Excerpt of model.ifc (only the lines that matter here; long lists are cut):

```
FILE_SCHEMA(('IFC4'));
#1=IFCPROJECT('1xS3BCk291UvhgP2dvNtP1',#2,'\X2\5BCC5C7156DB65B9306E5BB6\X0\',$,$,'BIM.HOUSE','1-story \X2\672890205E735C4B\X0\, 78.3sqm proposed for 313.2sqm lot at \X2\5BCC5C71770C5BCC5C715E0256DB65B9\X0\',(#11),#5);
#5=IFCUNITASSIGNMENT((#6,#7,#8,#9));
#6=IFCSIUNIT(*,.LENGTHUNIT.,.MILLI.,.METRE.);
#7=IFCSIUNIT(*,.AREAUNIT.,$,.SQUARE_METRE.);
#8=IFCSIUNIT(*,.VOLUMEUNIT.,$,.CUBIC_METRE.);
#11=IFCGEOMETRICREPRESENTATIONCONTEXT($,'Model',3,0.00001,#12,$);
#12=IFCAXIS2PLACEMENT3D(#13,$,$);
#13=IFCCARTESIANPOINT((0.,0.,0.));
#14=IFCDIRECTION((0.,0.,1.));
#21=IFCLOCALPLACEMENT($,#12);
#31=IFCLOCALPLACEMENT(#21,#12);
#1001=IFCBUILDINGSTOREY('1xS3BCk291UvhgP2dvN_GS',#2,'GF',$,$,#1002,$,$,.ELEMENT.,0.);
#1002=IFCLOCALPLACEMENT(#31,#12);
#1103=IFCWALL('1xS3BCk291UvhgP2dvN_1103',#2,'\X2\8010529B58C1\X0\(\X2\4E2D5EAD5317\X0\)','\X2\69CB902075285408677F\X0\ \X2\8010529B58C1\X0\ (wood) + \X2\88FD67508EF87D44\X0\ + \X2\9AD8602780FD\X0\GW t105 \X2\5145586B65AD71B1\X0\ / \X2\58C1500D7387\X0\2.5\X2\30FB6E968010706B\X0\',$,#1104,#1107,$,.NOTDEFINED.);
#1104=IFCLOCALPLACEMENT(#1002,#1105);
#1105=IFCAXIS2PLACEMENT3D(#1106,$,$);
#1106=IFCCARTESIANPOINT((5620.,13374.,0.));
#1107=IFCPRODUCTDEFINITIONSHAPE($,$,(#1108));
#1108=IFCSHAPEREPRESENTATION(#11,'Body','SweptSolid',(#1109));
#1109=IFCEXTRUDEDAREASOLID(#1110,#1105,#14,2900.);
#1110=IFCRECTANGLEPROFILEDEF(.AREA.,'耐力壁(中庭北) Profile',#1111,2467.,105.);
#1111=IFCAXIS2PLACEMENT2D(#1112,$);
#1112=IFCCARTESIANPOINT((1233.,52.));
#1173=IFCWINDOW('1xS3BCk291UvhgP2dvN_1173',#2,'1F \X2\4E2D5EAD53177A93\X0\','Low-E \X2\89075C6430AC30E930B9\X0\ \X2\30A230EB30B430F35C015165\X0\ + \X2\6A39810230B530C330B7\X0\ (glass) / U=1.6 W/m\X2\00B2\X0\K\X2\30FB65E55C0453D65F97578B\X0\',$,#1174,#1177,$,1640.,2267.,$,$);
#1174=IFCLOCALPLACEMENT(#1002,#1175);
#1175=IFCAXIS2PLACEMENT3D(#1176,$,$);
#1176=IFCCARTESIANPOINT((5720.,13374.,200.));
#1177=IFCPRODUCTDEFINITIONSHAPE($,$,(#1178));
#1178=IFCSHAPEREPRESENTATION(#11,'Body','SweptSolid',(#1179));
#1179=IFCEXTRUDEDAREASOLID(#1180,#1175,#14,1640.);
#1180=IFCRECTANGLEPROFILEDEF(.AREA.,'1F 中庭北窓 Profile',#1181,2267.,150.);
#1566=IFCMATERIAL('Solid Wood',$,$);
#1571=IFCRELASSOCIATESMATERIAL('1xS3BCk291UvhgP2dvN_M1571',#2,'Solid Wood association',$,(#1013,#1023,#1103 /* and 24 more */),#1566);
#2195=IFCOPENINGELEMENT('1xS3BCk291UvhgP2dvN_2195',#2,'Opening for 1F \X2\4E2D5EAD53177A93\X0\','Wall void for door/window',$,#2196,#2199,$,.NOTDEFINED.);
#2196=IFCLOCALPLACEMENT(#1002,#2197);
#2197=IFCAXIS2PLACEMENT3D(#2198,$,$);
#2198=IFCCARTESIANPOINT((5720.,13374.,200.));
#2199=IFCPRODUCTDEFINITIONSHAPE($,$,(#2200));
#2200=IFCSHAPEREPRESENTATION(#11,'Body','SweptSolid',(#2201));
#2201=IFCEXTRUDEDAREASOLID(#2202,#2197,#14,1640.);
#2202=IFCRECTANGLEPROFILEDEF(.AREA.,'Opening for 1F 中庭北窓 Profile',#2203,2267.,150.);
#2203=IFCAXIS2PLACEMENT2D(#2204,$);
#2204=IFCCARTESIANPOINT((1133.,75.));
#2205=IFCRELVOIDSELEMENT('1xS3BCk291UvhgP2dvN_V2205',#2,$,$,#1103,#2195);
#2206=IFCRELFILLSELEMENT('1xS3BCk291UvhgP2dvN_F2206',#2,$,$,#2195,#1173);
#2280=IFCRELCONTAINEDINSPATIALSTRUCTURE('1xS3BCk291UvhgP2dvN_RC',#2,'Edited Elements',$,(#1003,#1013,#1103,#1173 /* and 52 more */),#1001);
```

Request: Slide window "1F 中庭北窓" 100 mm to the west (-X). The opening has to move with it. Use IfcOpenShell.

```python
import ifcopenshell
import ifcopenshell.api.geometry
import ifcopenshell.util.placement
import ifcopenshell.util.unit

model = ifcopenshell.open("model.ifc")
unit_scale = ifcopenshell.util.unit.calculate_unit_scale(model)

window = model.by_id(1173)
opening = window.FillsVoids[0].RelatingOpeningElement
wall = opening.VoidsElements[0].RelatingBuildingElement

wall_matrix = ifcopenshell.util.placement.get_local_placement(wall.ObjectPlacement)
shift = wall_matrix[:3, 0] * -0.1 / unit_scale
before = ifcopenshell.util.placement.get_local_placement(window.ObjectPlacement)[:3, 3].copy()

# The window is not placed relative to its opening, so move both.
for product in (opening, window):
    matrix = ifcopenshell.util.placement.get_local_placement(product.ObjectPlacement)
    matrix[:3, 3] += shift
    ifcopenshell.api.geometry.edit_object_placement(model, product=product, matrix=matrix, is_si=False)

after = ifcopenshell.util.placement.get_local_placement(window.ObjectPlacement)[:3, 3]
print("window moved by", (after - before).round(3) + 0.0)

model.write("model-out.ifc")
```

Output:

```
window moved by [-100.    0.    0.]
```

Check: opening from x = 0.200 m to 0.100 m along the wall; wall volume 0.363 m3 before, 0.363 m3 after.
